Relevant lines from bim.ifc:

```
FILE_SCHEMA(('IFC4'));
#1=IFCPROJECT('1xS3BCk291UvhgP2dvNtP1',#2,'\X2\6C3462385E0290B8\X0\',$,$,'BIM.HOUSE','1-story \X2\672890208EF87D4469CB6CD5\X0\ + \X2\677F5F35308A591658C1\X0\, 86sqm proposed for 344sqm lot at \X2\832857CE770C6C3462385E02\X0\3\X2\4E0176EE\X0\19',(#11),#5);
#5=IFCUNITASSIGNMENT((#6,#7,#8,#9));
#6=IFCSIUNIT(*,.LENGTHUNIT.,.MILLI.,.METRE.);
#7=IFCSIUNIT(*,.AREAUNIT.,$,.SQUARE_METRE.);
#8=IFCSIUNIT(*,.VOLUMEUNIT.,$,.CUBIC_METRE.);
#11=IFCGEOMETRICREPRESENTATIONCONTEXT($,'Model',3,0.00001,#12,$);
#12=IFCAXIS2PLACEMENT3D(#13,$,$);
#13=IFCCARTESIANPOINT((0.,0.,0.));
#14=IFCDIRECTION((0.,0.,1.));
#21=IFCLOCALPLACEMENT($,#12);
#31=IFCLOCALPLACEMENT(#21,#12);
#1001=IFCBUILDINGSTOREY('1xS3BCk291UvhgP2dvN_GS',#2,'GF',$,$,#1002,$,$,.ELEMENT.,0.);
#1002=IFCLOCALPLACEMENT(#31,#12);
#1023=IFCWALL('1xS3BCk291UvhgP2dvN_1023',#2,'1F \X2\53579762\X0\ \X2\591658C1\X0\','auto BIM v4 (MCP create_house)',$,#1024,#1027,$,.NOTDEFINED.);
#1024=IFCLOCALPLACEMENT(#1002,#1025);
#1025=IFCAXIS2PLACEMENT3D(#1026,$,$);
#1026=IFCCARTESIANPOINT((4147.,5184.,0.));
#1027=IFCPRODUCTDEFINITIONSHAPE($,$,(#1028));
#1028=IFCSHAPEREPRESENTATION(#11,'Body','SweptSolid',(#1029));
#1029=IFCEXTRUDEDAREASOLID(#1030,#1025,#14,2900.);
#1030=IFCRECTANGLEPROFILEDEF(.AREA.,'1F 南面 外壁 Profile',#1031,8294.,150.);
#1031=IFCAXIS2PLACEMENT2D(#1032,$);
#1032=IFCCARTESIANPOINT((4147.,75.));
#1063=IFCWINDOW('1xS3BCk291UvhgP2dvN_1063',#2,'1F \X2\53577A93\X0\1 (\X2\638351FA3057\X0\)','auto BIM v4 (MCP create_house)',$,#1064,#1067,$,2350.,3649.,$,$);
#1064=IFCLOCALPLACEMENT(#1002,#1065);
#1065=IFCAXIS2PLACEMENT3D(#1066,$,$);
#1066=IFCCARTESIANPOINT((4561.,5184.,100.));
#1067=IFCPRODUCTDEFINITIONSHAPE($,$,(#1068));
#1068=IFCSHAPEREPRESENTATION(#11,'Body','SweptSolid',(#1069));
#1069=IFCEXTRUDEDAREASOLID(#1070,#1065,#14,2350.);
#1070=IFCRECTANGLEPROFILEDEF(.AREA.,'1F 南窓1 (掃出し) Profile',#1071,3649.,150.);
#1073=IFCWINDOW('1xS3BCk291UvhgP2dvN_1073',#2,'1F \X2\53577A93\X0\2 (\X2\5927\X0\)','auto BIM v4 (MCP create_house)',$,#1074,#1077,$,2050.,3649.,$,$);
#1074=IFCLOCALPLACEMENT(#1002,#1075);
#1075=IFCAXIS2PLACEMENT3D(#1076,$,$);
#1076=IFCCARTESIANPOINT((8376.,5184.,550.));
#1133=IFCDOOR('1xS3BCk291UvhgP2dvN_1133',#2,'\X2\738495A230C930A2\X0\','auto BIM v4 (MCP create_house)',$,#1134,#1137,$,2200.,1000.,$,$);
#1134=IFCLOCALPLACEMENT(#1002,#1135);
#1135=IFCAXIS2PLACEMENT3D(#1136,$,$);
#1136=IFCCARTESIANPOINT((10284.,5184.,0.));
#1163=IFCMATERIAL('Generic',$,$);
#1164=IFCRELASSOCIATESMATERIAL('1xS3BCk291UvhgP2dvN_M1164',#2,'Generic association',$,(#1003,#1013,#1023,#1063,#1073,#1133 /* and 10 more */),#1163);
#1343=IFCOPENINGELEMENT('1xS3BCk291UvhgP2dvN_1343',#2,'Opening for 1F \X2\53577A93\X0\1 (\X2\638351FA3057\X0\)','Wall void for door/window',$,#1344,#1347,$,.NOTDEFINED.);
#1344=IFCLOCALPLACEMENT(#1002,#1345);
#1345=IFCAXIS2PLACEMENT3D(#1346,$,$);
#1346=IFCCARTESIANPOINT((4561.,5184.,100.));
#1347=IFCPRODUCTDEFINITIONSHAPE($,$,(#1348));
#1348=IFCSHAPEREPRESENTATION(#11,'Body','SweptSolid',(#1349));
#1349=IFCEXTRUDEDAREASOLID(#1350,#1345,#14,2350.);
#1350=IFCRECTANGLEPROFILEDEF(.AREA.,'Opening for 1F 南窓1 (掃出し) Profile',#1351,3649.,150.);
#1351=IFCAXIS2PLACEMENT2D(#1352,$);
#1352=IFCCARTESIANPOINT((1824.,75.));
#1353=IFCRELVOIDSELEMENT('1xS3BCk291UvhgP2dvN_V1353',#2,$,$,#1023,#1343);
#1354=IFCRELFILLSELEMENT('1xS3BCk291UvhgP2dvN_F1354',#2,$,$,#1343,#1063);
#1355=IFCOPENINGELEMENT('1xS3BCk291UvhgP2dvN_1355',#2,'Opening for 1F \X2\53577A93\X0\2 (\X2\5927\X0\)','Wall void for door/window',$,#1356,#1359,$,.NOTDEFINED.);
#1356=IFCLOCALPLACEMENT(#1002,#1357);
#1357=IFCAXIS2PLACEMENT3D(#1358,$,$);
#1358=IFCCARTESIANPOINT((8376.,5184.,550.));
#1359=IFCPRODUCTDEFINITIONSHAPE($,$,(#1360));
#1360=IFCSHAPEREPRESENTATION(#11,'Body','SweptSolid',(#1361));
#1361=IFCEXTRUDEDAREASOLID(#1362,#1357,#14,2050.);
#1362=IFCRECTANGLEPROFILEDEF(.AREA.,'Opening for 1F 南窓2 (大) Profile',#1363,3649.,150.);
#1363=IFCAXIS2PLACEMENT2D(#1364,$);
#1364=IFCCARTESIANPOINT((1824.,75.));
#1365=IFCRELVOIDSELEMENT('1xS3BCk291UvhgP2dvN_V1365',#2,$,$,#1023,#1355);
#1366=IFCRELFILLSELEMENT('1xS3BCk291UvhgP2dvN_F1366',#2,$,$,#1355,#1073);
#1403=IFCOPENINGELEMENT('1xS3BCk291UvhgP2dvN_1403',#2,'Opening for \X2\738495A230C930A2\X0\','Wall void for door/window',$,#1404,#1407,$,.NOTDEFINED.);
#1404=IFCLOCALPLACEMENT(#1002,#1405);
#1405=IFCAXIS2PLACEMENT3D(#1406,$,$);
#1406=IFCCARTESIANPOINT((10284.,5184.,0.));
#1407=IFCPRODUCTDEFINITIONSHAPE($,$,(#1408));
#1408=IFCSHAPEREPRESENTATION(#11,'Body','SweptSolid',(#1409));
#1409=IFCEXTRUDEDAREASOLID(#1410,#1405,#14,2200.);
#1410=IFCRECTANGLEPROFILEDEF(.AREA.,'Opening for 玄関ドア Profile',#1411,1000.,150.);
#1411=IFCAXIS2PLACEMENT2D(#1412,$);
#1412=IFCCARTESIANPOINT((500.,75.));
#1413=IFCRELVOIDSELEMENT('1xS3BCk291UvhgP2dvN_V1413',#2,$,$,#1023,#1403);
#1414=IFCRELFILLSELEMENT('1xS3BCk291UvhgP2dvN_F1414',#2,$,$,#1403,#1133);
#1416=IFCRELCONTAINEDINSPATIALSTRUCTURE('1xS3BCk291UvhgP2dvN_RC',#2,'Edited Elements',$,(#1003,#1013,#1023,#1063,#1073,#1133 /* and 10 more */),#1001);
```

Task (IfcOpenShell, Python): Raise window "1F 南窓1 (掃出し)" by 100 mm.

```python
import numpy as np
import ifcopenshell
import ifcopenshell.api.geometry
import ifcopenshell.util.placement
import ifcopenshell.util.unit

model = ifcopenshell.open("bim.ifc")
unit_scale = ifcopenshell.util.unit.calculate_unit_scale(model)

window = model.by_guid("1xS3BCk291UvhgP2dvN_1063")
opening = window.FillsVoids[0].RelatingOpeningElement
dz = 100.0

shift = np.array([0.0, 0.0, dz])
# The window is not placed relative to its opening, so move both.
for product in (opening, window):
    matrix = ifcopenshell.util.placement.get_local_placement(product.ObjectPlacement)
    matrix[:3, 3] += shift
    ifcopenshell.api.geometry.edit_object_placement(model, product=product, matrix=matrix, is_si=False)

print(f"moved by {dz * unit_scale:+.3f} m")

model.write("bim_v2.ifc")
```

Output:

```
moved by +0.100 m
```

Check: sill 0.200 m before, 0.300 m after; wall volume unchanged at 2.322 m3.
